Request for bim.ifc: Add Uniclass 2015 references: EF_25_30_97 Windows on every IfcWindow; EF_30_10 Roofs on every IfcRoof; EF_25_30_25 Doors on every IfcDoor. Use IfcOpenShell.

First a look at what the model holds.

```python
import ifcopenshell

model = ifcopenshell.open("bim.ifc")
print(model.schema)
print("classifications:", [c.Name for c in model.by_type("IfcClassification")])
for ifc_class in ("IfcDoor", "IfcRoof", "IfcStair", "IfcWall", "IfcWindow"):
    print(ifc_class, len(model.by_type(ifc_class)))
```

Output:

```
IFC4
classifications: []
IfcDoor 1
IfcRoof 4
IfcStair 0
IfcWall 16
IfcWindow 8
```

```python
import ifcopenshell
import ifcopenshell.api.classification

model = ifcopenshell.open("bim.ifc")

system = ifcopenshell.api.classification.add_classification(model, classification="Uniclass 2015")

codes = {
    "IfcWindow": ("EF_25_30_97", "Windows"),
    "IfcRoof": ("EF_30_10", "Roofs"),
    "IfcDoor": ("EF_25_30_25", "Doors"),
}
for ifc_class, (code, name) in codes.items():
    products = model.by_type(ifc_class)
    ifcopenshell.api.classification.add_reference(
        model, products=products, classification=system, identification=code, name=name
    )
    print(code, len(products))

model.write("bim_v2.ifc")
```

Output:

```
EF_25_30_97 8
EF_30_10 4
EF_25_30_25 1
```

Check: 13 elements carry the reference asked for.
